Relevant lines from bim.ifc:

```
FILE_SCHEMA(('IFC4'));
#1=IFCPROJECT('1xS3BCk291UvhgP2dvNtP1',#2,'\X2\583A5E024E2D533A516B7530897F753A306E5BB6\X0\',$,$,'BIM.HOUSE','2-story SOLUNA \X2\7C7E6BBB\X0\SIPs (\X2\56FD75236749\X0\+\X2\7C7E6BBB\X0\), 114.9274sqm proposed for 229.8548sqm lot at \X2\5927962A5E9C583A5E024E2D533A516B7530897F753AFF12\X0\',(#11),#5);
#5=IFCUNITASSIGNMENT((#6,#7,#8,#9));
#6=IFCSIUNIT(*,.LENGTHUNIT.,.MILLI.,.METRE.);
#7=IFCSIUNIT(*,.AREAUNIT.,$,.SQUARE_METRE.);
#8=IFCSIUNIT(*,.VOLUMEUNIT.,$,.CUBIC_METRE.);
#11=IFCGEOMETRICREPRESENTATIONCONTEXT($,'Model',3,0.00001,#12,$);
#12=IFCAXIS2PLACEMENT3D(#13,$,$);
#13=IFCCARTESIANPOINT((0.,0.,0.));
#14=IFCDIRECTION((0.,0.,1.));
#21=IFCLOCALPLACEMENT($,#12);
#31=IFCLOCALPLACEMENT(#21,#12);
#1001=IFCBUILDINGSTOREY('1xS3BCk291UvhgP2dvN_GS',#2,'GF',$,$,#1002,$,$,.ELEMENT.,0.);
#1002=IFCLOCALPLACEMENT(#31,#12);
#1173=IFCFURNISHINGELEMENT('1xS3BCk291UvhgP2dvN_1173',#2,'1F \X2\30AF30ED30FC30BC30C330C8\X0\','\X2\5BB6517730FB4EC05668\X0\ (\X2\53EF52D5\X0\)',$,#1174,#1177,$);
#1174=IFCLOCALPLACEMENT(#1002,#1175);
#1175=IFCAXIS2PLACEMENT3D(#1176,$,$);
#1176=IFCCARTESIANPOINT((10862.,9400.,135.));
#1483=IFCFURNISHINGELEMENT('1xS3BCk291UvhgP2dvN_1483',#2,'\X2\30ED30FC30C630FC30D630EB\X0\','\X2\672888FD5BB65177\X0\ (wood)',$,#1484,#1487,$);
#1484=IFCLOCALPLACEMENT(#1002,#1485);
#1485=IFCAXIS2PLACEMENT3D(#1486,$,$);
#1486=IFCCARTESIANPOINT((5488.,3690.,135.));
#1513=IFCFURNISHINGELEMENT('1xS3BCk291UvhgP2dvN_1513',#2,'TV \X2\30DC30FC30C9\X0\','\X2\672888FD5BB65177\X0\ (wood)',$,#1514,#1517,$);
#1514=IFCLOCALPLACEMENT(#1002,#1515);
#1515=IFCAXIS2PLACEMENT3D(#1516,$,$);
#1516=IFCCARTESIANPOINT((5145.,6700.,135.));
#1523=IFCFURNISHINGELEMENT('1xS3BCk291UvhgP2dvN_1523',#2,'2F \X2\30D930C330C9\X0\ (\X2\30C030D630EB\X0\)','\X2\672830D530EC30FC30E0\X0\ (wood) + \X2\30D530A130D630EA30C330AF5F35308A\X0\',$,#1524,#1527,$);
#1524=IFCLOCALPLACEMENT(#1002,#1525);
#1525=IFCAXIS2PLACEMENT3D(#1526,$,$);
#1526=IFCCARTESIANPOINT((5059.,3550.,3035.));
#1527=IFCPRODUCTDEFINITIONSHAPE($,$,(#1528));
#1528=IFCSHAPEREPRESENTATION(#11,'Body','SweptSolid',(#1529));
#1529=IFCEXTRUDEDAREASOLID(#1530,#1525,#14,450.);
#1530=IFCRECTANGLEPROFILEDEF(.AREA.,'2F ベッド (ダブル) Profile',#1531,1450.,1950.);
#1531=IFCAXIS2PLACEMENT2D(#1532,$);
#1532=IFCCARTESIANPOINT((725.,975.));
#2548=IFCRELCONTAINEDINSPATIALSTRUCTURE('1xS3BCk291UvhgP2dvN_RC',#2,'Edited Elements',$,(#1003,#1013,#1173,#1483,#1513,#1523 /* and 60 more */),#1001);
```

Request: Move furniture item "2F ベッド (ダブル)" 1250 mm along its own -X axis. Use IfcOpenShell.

```python
import ifcopenshell
import ifcopenshell.api.geometry
import ifcopenshell.util.placement
import ifcopenshell.util.unit

model = ifcopenshell.open("bim.ifc")
unit_scale = ifcopenshell.util.unit.calculate_unit_scale(model)

item = model.by_id(1523)
matrix = ifcopenshell.util.placement.get_local_placement(item.ObjectPlacement)
matrix[:3, 3] -= matrix[:3, 0] * 1.25 / unit_scale
ifcopenshell.api.geometry.edit_object_placement(model, product=item, matrix=matrix, is_si=False)

print(ifcopenshell.util.placement.get_local_placement(item.ObjectPlacement).round(3) + 0.0)

model.write("bim_v2.ifc")
```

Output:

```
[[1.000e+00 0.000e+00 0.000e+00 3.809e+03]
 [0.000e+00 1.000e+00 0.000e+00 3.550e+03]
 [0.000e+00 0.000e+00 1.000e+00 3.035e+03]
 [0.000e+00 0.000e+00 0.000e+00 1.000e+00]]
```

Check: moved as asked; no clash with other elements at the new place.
